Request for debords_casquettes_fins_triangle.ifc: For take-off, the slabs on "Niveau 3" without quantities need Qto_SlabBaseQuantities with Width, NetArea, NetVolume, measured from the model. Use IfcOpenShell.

First a look at what the model holds.

```python
import ifcopenshell
import ifcopenshell.util.element
import ifcopenshell.util.unit

model = ifcopenshell.open("debords_casquettes_fins_triangle.ifc")
print(model.schema)
for unit_type in ("LENGTHUNIT", "AREAUNIT", "VOLUMEUNIT"):
    print(unit_type, ifcopenshell.util.unit.calculate_unit_scale(model, unit_type))
storey = next(s for s in model.by_type("IfcBuildingStorey") if s.Name == "Niveau 3")
slabs = [e for e in ifcopenshell.util.element.get_decomposition(storey) if e.is_a("IfcSlab")]
for e in sorted(slabs, key=lambda e: e.id()):
    print(e.id(), e.is_a(), e.Name, list(ifcopenshell.util.element.get_psets(e, qtos_only=True)), sep=" | ")
```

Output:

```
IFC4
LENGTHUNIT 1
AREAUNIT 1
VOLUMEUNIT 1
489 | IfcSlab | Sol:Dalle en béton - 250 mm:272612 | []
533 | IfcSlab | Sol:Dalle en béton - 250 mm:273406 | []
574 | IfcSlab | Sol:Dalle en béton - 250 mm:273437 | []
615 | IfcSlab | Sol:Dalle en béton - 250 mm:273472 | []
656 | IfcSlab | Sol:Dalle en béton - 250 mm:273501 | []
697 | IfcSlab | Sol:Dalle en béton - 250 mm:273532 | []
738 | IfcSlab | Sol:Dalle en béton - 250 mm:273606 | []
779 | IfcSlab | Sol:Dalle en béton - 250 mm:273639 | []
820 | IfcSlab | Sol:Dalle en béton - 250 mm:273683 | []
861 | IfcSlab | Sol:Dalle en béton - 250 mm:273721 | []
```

```python
import ifcopenshell
import ifcopenshell.api.pset
import ifcopenshell.geom
import ifcopenshell.util.element
import ifcopenshell.util.shape
import ifcopenshell.util.unit

model = ifcopenshell.open("debords_casquettes_fins_triangle.ifc")
unit_scale = ifcopenshell.util.unit.calculate_unit_scale(model)
area_scale = ifcopenshell.util.unit.calculate_unit_scale(model, "AREAUNIT")
volume_scale = ifcopenshell.util.unit.calculate_unit_scale(model, "VOLUMEUNIT")
settings = ifcopenshell.geom.settings()

storey = next(s for s in model.by_type("IfcBuildingStorey") if s.Name == "Niveau 3")
slabs = [e for e in ifcopenshell.util.element.get_decomposition(storey) if e.is_a("IfcSlab")]

for e in sorted(slabs, key=lambda e: e.id()):
    if ifcopenshell.util.element.get_psets(e, qtos_only=True, should_inherit=False):
        continue
    # Geometry comes back in metres, in the element's own axes.
    shape = ifcopenshell.geom.create_shape(settings, e)
    values = {
        "Width": ifcopenshell.util.shape.get_z(shape.geometry) / unit_scale,
        "NetArea": ifcopenshell.util.shape.get_footprint_area(shape.geometry) / area_scale,
        "NetVolume": ifcopenshell.util.shape.get_volume(shape.geometry) / volume_scale,
    }
    qto = ifcopenshell.api.pset.add_qto(model, product=e, name="Qto_SlabBaseQuantities")
    ifcopenshell.api.pset.edit_qto(model, qto=qto, properties=values)
    print(e.id(), {k: round(v, 3) for k, v in values.items()})

model.write("debords_casquettes_fins_triangle-out.ifc")
```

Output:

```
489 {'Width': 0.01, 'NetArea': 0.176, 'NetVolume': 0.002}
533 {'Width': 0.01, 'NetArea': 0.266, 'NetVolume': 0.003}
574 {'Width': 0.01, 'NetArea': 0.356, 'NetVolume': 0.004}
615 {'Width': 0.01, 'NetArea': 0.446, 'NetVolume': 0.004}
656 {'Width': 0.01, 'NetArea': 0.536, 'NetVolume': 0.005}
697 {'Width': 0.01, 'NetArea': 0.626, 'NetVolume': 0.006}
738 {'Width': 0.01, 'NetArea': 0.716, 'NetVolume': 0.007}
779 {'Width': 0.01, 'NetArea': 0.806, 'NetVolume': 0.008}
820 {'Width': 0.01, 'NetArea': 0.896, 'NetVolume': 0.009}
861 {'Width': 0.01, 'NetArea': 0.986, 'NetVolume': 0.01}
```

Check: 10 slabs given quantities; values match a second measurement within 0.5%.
